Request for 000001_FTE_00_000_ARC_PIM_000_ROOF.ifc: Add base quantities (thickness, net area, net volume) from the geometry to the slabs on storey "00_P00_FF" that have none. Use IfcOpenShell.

First a look at what the model holds.

```python
import ifcopenshell
import ifcopenshell.util.element
import ifcopenshell.util.unit

model = ifcopenshell.open("000001_FTE_00_000_ARC_PIM_000_ROOF.ifc")
print(model.schema)
for unit_type in ("LENGTHUNIT", "AREAUNIT", "VOLUMEUNIT"):
    print(unit_type, ifcopenshell.util.unit.calculate_unit_scale(model, unit_type))
storey = next(s for s in model.by_type("IfcBuildingStorey") if s.Name == "00_P00_FF")
slabs = [e for e in ifcopenshell.util.element.get_decomposition(storey) if e.is_a("IfcSlab")]
for e in sorted(slabs, key=lambda e: e.id()):
    print(e.id(), e.is_a(), e.Name, list(ifcopenshell.util.element.get_psets(e, qtos_only=True)), sep=" | ")
```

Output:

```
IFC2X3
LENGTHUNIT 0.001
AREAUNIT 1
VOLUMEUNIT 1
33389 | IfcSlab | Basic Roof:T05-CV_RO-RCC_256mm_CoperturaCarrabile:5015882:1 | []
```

```python
import ifcopenshell
import ifcopenshell.api.pset
import ifcopenshell.geom
import ifcopenshell.util.element
import ifcopenshell.util.shape
import ifcopenshell.util.unit

model = ifcopenshell.open("000001_FTE_00_000_ARC_PIM_000_ROOF.ifc")
unit_scale = ifcopenshell.util.unit.calculate_unit_scale(model)
area_scale = ifcopenshell.util.unit.calculate_unit_scale(model, "AREAUNIT")
volume_scale = ifcopenshell.util.unit.calculate_unit_scale(model, "VOLUMEUNIT")
settings = ifcopenshell.geom.settings()

storey = next(s for s in model.by_type("IfcBuildingStorey") if s.Name == "00_P00_FF")
slabs = [e for e in ifcopenshell.util.element.get_decomposition(storey) if e.is_a("IfcSlab")]

for e in sorted(slabs, key=lambda e: e.id()):
    if ifcopenshell.util.element.get_psets(e, qtos_only=True, should_inherit=False):
        continue
    # Geometry comes back in metres, in the element's own axes.
    shape = ifcopenshell.geom.create_shape(settings, e)
    values = {
        "Width": ifcopenshell.util.shape.get_z(shape.geometry) / unit_scale,
        "NetArea": ifcopenshell.util.shape.get_footprint_area(shape.geometry) / area_scale,
        "NetVolume": ifcopenshell.util.shape.get_volume(shape.geometry) / volume_scale,
    }
    qto = ifcopenshell.api.pset.add_qto(model, product=e, name="BaseQuantities")
    ifcopenshell.api.pset.edit_qto(model, qto=qto, properties=values)
    print(e.id(), {k: round(v, 3) for k, v in values.items()})

model.write("000001_FTE_00_000_ARC_PIM_000_ROOF_rev.ifc")
```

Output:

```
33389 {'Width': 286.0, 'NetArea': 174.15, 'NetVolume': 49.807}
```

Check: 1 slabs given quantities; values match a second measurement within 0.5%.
